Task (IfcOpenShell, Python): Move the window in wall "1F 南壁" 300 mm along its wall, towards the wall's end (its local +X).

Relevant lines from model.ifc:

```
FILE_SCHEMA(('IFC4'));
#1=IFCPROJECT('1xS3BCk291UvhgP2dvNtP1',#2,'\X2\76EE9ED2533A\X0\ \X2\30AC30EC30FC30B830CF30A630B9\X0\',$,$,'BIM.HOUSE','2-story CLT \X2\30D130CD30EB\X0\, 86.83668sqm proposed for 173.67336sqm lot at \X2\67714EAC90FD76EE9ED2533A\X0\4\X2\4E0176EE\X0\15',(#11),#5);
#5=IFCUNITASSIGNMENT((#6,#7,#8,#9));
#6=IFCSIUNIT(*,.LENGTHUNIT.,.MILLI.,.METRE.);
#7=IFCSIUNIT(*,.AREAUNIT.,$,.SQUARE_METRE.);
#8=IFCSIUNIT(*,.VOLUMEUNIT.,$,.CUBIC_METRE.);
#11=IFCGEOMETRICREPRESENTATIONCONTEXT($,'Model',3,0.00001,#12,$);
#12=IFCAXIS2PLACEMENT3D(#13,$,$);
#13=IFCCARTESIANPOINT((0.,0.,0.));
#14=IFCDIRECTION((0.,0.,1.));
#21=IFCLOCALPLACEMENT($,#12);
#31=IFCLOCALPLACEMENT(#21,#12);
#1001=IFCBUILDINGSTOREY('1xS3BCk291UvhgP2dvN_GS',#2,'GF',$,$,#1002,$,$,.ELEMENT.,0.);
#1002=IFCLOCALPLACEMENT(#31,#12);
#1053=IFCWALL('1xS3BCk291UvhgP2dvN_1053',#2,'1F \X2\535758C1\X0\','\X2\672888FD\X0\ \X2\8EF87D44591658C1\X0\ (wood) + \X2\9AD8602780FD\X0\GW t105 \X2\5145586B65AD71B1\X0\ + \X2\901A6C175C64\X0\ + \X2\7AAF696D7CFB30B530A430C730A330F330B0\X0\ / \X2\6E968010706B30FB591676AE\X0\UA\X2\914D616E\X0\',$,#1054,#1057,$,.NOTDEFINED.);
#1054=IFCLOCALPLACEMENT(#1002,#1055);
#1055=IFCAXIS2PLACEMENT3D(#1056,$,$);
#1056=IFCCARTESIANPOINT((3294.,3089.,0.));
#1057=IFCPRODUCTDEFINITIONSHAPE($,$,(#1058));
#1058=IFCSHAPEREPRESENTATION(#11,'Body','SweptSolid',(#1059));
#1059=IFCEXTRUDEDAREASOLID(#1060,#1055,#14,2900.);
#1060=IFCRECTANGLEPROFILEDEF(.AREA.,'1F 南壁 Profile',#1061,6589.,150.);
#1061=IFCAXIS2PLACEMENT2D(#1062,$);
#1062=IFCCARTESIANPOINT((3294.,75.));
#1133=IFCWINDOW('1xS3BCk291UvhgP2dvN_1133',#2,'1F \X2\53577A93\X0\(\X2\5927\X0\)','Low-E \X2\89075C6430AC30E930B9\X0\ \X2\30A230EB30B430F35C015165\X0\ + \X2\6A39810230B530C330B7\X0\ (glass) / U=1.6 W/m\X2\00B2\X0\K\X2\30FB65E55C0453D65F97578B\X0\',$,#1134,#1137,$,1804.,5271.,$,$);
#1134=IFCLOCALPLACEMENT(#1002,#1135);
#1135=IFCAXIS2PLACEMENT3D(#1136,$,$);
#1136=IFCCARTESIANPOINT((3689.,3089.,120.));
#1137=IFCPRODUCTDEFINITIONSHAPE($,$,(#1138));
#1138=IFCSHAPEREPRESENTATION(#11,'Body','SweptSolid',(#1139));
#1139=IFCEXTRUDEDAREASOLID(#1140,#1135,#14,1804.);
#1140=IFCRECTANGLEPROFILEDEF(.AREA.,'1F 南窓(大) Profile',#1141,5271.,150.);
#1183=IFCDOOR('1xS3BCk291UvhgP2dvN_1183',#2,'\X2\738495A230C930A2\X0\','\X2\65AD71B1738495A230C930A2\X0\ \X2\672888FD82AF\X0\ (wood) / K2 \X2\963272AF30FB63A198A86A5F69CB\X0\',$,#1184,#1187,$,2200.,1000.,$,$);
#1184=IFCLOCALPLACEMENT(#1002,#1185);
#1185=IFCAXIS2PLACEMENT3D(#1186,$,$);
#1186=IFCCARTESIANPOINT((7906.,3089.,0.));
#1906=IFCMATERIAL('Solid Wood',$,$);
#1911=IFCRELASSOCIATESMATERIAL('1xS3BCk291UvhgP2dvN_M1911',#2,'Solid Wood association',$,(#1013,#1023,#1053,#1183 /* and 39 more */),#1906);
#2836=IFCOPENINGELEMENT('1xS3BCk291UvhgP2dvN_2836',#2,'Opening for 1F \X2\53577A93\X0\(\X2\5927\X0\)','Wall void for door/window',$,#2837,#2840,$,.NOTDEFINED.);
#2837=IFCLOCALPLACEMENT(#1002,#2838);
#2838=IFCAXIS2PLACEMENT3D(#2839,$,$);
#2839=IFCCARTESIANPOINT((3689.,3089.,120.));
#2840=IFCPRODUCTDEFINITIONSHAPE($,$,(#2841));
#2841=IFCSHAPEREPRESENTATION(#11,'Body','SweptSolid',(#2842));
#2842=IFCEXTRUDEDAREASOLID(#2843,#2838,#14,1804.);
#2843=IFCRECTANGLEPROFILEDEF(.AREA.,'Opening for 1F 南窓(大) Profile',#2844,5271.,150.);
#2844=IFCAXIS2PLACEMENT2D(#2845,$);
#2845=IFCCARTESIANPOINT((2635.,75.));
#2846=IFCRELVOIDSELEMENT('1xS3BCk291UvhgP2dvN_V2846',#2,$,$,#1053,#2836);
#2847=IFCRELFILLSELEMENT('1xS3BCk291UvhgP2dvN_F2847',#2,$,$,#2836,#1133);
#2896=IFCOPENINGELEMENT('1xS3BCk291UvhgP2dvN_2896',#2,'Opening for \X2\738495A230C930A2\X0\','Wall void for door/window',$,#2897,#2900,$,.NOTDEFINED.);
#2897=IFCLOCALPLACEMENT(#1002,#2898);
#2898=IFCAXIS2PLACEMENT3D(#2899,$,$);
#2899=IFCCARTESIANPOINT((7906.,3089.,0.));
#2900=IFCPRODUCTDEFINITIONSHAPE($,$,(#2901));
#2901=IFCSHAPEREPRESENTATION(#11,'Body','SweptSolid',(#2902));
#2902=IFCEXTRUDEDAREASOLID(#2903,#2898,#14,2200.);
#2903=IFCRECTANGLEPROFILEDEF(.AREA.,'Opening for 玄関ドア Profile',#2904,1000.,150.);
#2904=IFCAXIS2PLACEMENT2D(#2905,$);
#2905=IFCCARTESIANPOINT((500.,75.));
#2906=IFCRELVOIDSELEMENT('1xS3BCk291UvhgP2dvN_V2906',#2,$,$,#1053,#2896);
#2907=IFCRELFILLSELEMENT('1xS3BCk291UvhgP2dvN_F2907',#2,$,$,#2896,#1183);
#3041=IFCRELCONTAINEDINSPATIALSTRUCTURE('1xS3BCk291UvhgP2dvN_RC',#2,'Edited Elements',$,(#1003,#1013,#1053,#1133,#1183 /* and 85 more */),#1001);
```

```python
import ifcopenshell
import ifcopenshell.api.geometry
import ifcopenshell.util.placement

model = ifcopenshell.open("model.ifc")

window = model.by_guid("1xS3BCk291UvhgP2dvN_1133")
opening = window.FillsVoids[0].RelatingOpeningElement
wall = opening.VoidsElements[0].RelatingBuildingElement

wall_matrix = ifcopenshell.util.placement.get_local_placement(wall.ObjectPlacement)
shift = wall_matrix[:3, 0] * 300.0
before = ifcopenshell.util.placement.get_local_placement(window.ObjectPlacement)[:3, 3].copy()

# The window is not placed relative to its opening, so move both.
for product in (opening, window):
    matrix = ifcopenshell.util.placement.get_local_placement(product.ObjectPlacement)
    matrix[:3, 3] += shift
    ifcopenshell.api.geometry.edit_object_placement(model, product=product, matrix=matrix, is_si=False)

after = ifcopenshell.util.placement.get_local_placement(window.ObjectPlacement)[:3, 3]
print("window moved by", (after - before).round(3) + 0.0)

model.write("model_updated.ifc")
```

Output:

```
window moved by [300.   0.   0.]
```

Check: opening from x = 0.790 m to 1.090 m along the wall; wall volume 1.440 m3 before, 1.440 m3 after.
